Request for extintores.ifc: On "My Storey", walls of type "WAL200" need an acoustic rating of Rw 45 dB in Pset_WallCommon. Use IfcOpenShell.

First a look at what the model holds.

```python
import ifcopenshell
import ifcopenshell.util.element

model = ifcopenshell.open("extintores.ifc")
print(model.schema)
storey = next(s for s in model.by_type("IfcBuildingStorey") if s.Name == "My Storey")
walls = [e for e in ifcopenshell.util.element.get_decomposition(storey) if e.is_a("IfcWall")]
seen = {}
for e in walls:
    element_type = ifcopenshell.util.element.get_type(e)
    key = (element_type.Name if element_type != e and element_type else None, ifcopenshell.util.element.get_pset(e, "Pset_WallCommon", "AcousticRating"))
    seen[key] = seen.get(key, 0) + 1
for (name, value), count in sorted(seen.items(), key=str):
    print(count, "x", name, "|", value)
```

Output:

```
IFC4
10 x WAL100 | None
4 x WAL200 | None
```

```python
import ifcopenshell
import ifcopenshell.api.pset
import ifcopenshell.util.element

model = ifcopenshell.open("extintores.ifc")

storey = next(s for s in model.by_type("IfcBuildingStorey") if s.Name == "My Storey")
walls = [e for e in ifcopenshell.util.element.get_decomposition(storey) if e.is_a("IfcWall")]

count = 0
for e in walls:
    element_type = ifcopenshell.util.element.get_type(e)
    if element_type in (None, e) or element_type.Name != "WAL200":
        continue
    # add_pset returns the element's existing set when there is one.
    pset = ifcopenshell.api.pset.add_pset(model, product=e, name="Pset_WallCommon")
    ifcopenshell.api.pset.edit_pset(model, pset=pset, properties={"AcousticRating": "Rw 45 dB"})
    count += 1

print(count, "walls updated")

model.write("extintores_v2.ifc")
```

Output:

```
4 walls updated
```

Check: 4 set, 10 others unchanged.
